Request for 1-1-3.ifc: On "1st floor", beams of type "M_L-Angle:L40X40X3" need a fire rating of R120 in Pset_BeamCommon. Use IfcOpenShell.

First a look at what the model holds.

```python
import ifcopenshell
import ifcopenshell.util.element

model = ifcopenshell.open("1-1-3.ifc")
print(model.schema)
storey = next(s for s in model.by_type("IfcBuildingStorey") if s.Name == "1st floor")
beams = [e for e in ifcopenshell.util.element.get_decomposition(storey) if e.is_a("IfcBeam")]
seen = {}
for e in beams:
    element_type = ifcopenshell.util.element.get_type(e)
    key = (element_type.Name if element_type != e and element_type else None, ifcopenshell.util.element.get_pset(e, "Pset_BeamCommon", "FireRating"))
    seen[key] = seen.get(key, 0) + 1
for (name, value), count in sorted(seen.items(), key=str):
    print(count, "x", name, "|", value)
```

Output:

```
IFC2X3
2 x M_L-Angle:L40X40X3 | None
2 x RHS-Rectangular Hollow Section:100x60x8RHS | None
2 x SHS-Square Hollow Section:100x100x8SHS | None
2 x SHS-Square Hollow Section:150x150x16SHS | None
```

```python
import ifcopenshell
import ifcopenshell.api.pset
import ifcopenshell.util.element

model = ifcopenshell.open("1-1-3.ifc")

storey = next(s for s in model.by_type("IfcBuildingStorey") if s.Name == "1st floor")
beams = [e for e in ifcopenshell.util.element.get_decomposition(storey) if e.is_a("IfcBeam")]

count = 0
for e in beams:
    element_type = ifcopenshell.util.element.get_type(e)
    if element_type in (None, e) or element_type.Name != "M_L-Angle:L40X40X3":
        continue
    # add_pset returns the element's existing set when there is one.
    pset = ifcopenshell.api.pset.add_pset(model, product=e, name="Pset_BeamCommon")
    ifcopenshell.api.pset.edit_pset(model, pset=pset, properties={"FireRating": "R120"})
    count += 1

print(count, "beams updated")

model.write("1-1-3_updated.ifc")
```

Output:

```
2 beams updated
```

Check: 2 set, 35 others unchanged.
